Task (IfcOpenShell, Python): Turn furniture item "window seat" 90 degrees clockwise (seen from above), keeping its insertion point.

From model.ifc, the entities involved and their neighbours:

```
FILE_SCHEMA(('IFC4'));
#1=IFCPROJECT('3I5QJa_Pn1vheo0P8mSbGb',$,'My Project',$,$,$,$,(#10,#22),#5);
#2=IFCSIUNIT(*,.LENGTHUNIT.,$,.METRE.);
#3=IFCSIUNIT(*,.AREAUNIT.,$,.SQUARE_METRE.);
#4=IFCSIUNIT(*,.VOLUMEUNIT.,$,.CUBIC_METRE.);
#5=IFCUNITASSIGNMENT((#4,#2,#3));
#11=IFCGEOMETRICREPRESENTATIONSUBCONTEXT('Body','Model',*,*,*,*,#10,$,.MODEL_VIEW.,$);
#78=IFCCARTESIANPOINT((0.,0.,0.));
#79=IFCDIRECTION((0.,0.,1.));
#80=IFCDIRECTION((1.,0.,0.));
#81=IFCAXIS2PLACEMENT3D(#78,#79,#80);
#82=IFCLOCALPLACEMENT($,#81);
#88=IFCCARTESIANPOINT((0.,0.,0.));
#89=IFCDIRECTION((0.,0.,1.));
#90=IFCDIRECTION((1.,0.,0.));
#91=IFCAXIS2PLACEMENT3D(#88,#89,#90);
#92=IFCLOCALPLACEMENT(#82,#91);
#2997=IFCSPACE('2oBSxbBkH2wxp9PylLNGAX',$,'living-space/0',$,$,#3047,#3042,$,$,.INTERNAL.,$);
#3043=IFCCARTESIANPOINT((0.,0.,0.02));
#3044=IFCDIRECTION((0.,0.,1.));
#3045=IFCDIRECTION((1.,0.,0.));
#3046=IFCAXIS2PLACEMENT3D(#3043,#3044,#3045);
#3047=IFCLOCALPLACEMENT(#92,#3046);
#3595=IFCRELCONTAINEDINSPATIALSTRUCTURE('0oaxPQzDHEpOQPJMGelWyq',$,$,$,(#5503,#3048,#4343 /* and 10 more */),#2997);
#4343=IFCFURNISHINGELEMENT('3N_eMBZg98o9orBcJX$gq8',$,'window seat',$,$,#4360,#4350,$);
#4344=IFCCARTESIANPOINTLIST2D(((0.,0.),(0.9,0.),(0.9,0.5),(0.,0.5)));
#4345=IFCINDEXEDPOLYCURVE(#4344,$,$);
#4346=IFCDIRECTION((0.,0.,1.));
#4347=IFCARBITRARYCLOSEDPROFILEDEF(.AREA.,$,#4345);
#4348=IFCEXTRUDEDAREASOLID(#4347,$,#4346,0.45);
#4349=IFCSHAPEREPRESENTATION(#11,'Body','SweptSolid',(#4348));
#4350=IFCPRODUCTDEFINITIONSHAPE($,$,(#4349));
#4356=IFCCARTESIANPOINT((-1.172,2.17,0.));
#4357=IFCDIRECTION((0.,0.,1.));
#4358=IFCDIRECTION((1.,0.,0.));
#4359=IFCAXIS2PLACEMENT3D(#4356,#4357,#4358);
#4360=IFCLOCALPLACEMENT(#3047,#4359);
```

```python
import ifcopenshell
import ifcopenshell.api.geometry
import ifcopenshell.util.placement

model = ifcopenshell.open("model.ifc")

item = model.by_id(4343)
matrix = ifcopenshell.util.placement.get_local_placement(item.ObjectPlacement)
matrix = matrix @ ifcopenshell.util.placement.rotation(-90, "Z")
ifcopenshell.api.geometry.edit_object_placement(model, product=item, matrix=matrix, is_si=False)

print(ifcopenshell.util.placement.get_local_placement(item.ObjectPlacement).round(3) + 0.0)

model.write("model-out.ifc")
```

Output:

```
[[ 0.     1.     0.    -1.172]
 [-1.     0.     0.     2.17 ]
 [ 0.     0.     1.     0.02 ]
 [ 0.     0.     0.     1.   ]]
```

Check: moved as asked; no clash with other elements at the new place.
